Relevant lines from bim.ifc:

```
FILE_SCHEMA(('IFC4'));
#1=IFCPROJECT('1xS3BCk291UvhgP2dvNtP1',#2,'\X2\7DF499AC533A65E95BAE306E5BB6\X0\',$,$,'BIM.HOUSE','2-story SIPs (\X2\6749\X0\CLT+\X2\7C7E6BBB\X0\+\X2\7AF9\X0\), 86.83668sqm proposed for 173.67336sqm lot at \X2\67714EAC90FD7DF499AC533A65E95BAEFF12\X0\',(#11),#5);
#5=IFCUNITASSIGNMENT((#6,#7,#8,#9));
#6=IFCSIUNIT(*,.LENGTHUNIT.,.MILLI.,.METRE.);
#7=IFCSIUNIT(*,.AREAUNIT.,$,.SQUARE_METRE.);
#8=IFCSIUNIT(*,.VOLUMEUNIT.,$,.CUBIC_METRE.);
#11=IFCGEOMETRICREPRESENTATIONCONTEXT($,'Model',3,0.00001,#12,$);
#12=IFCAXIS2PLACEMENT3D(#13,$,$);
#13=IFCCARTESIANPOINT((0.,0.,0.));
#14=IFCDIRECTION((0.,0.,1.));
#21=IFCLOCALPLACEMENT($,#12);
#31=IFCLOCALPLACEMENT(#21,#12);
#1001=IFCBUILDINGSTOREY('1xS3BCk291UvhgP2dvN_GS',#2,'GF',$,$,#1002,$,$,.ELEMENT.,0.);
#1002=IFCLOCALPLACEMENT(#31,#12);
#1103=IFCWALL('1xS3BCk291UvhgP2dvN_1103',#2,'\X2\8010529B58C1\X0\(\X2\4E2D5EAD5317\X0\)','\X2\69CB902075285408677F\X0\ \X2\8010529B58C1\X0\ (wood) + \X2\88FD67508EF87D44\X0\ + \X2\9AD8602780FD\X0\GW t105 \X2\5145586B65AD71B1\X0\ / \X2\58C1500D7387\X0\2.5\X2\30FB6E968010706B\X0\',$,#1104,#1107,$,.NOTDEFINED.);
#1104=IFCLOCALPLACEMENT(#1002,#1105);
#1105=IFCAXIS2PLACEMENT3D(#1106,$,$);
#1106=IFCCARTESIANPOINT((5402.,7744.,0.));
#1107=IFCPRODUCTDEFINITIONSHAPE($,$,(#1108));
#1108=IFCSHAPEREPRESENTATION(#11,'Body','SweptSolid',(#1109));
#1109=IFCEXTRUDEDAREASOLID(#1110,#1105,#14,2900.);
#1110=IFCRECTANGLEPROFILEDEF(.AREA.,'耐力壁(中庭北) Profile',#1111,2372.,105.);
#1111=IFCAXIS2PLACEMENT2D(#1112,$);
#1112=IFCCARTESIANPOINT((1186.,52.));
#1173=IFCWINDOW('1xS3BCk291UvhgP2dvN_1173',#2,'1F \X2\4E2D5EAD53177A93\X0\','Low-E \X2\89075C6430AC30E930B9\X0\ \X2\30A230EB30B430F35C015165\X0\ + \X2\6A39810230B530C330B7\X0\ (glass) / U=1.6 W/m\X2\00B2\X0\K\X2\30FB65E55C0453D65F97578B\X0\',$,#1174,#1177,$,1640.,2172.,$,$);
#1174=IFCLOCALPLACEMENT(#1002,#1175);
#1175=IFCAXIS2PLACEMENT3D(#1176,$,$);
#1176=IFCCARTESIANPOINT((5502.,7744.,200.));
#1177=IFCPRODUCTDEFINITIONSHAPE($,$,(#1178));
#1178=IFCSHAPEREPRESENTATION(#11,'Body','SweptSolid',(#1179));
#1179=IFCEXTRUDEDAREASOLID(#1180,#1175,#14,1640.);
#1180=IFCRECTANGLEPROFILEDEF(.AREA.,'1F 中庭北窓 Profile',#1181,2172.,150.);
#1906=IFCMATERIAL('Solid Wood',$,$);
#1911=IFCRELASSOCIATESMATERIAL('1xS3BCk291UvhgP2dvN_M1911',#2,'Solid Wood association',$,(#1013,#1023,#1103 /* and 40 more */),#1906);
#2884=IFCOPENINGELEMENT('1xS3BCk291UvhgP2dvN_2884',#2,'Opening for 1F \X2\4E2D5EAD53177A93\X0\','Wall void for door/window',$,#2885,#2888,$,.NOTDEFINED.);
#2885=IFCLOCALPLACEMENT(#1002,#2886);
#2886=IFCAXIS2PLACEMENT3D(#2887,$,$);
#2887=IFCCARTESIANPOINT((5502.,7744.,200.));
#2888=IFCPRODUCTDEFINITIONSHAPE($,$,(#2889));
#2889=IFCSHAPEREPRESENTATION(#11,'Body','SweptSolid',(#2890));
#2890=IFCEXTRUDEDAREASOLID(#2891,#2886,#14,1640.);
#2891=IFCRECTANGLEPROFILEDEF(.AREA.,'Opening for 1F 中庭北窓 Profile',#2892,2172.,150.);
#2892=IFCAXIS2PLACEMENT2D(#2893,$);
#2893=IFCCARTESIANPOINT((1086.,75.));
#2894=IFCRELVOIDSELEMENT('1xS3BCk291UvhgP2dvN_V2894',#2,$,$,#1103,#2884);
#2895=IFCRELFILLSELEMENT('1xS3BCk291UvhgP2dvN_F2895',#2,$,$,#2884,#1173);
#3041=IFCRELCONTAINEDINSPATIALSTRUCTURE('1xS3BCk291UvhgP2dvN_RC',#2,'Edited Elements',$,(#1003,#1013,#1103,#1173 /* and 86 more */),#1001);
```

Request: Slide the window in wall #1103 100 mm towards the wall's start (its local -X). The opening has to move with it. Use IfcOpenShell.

```python
import ifcopenshell
import ifcopenshell.api.geometry
import ifcopenshell.util.placement

model = ifcopenshell.open("bim.ifc")

window = model.by_guid("1xS3BCk291UvhgP2dvN_1173")
opening = window.FillsVoids[0].RelatingOpeningElement
wall = opening.VoidsElements[0].RelatingBuildingElement

wall_matrix = ifcopenshell.util.placement.get_local_placement(wall.ObjectPlacement)
shift = wall_matrix[:3, 0] * -100.0
before = ifcopenshell.util.placement.get_local_placement(window.ObjectPlacement)[:3, 3].copy()

# The window is not placed relative to its opening, so move both.
for product in (opening, window):
    matrix = ifcopenshell.util.placement.get_local_placement(product.ObjectPlacement)
    matrix[:3, 3] += shift
    ifcopenshell.api.geometry.edit_object_placement(model, product=product, matrix=matrix, is_si=False)

after = ifcopenshell.util.placement.get_local_placement(window.ObjectPlacement)[:3, 3]
print("window moved by", (after - before).round(3) + 0.0)

model.write("bim-out.ifc")
```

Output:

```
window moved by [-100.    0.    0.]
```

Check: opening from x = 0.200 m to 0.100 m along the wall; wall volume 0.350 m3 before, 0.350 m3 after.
